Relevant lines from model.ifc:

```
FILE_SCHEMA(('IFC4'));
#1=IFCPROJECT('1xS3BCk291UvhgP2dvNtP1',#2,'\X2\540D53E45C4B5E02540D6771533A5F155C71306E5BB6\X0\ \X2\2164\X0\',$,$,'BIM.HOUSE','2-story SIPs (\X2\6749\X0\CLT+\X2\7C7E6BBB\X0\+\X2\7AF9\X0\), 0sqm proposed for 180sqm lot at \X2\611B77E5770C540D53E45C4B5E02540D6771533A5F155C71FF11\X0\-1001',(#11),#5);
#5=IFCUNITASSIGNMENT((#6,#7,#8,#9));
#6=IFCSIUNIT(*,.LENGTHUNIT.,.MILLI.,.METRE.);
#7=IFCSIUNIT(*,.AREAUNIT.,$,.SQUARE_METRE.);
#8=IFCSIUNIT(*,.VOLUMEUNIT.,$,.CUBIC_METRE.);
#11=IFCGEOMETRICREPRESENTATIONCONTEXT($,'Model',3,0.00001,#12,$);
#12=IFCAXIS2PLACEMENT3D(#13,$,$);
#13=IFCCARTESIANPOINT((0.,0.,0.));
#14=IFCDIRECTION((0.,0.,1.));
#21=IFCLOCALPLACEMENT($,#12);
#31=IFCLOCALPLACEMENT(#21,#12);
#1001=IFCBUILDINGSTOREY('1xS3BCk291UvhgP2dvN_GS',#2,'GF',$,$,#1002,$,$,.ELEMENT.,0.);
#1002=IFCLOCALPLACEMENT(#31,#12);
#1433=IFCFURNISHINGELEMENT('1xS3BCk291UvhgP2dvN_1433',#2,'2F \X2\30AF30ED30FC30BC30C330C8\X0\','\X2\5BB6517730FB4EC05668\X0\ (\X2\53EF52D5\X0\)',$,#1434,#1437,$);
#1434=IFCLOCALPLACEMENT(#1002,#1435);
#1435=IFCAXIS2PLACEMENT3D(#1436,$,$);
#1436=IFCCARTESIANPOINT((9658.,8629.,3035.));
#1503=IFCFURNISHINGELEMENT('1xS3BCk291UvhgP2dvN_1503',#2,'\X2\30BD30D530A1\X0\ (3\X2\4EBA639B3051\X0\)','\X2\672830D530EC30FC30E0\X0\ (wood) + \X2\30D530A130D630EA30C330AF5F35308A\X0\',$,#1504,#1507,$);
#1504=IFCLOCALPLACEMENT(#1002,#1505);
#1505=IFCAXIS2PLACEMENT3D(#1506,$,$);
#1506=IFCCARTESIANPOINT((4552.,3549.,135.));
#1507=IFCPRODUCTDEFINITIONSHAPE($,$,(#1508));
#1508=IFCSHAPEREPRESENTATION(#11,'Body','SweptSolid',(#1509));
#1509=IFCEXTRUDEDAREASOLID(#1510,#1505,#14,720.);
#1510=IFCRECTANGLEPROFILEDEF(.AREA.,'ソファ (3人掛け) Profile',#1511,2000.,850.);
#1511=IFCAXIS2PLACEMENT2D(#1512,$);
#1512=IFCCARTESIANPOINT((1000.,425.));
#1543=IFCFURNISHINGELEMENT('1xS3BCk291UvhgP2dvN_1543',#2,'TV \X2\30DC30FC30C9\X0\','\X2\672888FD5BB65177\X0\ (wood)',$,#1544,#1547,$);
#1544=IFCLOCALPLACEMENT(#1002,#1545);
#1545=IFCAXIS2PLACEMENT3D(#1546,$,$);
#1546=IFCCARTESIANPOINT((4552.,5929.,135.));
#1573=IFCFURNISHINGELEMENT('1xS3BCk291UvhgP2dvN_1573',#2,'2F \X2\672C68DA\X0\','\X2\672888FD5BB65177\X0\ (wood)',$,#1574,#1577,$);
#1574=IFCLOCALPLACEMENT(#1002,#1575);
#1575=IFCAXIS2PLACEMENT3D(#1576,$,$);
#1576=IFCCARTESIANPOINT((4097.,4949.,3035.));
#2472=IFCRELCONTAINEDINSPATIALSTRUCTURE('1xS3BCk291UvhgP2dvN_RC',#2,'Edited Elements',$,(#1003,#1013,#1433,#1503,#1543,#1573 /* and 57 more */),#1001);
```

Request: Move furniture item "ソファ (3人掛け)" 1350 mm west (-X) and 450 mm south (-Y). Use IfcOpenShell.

```python
import ifcopenshell
import ifcopenshell.api.geometry
import ifcopenshell.util.placement
import ifcopenshell.util.unit

model = ifcopenshell.open("model.ifc")
unit_scale = ifcopenshell.util.unit.calculate_unit_scale(model)

item = model.by_guid("1xS3BCk291UvhgP2dvN_1503")
matrix = ifcopenshell.util.placement.get_local_placement(item.ObjectPlacement)
matrix[0, 3] -= 1.35 / unit_scale
matrix[1, 3] -= 0.45 / unit_scale
ifcopenshell.api.geometry.edit_object_placement(model, product=item, matrix=matrix, is_si=False)

print(ifcopenshell.util.placement.get_local_placement(item.ObjectPlacement).round(3) + 0.0)

model.write("model-out.ifc")
```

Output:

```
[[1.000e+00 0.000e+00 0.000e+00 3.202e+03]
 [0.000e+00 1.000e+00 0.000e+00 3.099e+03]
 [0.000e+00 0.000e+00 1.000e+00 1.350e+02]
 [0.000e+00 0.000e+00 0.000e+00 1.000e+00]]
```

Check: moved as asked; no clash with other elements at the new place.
